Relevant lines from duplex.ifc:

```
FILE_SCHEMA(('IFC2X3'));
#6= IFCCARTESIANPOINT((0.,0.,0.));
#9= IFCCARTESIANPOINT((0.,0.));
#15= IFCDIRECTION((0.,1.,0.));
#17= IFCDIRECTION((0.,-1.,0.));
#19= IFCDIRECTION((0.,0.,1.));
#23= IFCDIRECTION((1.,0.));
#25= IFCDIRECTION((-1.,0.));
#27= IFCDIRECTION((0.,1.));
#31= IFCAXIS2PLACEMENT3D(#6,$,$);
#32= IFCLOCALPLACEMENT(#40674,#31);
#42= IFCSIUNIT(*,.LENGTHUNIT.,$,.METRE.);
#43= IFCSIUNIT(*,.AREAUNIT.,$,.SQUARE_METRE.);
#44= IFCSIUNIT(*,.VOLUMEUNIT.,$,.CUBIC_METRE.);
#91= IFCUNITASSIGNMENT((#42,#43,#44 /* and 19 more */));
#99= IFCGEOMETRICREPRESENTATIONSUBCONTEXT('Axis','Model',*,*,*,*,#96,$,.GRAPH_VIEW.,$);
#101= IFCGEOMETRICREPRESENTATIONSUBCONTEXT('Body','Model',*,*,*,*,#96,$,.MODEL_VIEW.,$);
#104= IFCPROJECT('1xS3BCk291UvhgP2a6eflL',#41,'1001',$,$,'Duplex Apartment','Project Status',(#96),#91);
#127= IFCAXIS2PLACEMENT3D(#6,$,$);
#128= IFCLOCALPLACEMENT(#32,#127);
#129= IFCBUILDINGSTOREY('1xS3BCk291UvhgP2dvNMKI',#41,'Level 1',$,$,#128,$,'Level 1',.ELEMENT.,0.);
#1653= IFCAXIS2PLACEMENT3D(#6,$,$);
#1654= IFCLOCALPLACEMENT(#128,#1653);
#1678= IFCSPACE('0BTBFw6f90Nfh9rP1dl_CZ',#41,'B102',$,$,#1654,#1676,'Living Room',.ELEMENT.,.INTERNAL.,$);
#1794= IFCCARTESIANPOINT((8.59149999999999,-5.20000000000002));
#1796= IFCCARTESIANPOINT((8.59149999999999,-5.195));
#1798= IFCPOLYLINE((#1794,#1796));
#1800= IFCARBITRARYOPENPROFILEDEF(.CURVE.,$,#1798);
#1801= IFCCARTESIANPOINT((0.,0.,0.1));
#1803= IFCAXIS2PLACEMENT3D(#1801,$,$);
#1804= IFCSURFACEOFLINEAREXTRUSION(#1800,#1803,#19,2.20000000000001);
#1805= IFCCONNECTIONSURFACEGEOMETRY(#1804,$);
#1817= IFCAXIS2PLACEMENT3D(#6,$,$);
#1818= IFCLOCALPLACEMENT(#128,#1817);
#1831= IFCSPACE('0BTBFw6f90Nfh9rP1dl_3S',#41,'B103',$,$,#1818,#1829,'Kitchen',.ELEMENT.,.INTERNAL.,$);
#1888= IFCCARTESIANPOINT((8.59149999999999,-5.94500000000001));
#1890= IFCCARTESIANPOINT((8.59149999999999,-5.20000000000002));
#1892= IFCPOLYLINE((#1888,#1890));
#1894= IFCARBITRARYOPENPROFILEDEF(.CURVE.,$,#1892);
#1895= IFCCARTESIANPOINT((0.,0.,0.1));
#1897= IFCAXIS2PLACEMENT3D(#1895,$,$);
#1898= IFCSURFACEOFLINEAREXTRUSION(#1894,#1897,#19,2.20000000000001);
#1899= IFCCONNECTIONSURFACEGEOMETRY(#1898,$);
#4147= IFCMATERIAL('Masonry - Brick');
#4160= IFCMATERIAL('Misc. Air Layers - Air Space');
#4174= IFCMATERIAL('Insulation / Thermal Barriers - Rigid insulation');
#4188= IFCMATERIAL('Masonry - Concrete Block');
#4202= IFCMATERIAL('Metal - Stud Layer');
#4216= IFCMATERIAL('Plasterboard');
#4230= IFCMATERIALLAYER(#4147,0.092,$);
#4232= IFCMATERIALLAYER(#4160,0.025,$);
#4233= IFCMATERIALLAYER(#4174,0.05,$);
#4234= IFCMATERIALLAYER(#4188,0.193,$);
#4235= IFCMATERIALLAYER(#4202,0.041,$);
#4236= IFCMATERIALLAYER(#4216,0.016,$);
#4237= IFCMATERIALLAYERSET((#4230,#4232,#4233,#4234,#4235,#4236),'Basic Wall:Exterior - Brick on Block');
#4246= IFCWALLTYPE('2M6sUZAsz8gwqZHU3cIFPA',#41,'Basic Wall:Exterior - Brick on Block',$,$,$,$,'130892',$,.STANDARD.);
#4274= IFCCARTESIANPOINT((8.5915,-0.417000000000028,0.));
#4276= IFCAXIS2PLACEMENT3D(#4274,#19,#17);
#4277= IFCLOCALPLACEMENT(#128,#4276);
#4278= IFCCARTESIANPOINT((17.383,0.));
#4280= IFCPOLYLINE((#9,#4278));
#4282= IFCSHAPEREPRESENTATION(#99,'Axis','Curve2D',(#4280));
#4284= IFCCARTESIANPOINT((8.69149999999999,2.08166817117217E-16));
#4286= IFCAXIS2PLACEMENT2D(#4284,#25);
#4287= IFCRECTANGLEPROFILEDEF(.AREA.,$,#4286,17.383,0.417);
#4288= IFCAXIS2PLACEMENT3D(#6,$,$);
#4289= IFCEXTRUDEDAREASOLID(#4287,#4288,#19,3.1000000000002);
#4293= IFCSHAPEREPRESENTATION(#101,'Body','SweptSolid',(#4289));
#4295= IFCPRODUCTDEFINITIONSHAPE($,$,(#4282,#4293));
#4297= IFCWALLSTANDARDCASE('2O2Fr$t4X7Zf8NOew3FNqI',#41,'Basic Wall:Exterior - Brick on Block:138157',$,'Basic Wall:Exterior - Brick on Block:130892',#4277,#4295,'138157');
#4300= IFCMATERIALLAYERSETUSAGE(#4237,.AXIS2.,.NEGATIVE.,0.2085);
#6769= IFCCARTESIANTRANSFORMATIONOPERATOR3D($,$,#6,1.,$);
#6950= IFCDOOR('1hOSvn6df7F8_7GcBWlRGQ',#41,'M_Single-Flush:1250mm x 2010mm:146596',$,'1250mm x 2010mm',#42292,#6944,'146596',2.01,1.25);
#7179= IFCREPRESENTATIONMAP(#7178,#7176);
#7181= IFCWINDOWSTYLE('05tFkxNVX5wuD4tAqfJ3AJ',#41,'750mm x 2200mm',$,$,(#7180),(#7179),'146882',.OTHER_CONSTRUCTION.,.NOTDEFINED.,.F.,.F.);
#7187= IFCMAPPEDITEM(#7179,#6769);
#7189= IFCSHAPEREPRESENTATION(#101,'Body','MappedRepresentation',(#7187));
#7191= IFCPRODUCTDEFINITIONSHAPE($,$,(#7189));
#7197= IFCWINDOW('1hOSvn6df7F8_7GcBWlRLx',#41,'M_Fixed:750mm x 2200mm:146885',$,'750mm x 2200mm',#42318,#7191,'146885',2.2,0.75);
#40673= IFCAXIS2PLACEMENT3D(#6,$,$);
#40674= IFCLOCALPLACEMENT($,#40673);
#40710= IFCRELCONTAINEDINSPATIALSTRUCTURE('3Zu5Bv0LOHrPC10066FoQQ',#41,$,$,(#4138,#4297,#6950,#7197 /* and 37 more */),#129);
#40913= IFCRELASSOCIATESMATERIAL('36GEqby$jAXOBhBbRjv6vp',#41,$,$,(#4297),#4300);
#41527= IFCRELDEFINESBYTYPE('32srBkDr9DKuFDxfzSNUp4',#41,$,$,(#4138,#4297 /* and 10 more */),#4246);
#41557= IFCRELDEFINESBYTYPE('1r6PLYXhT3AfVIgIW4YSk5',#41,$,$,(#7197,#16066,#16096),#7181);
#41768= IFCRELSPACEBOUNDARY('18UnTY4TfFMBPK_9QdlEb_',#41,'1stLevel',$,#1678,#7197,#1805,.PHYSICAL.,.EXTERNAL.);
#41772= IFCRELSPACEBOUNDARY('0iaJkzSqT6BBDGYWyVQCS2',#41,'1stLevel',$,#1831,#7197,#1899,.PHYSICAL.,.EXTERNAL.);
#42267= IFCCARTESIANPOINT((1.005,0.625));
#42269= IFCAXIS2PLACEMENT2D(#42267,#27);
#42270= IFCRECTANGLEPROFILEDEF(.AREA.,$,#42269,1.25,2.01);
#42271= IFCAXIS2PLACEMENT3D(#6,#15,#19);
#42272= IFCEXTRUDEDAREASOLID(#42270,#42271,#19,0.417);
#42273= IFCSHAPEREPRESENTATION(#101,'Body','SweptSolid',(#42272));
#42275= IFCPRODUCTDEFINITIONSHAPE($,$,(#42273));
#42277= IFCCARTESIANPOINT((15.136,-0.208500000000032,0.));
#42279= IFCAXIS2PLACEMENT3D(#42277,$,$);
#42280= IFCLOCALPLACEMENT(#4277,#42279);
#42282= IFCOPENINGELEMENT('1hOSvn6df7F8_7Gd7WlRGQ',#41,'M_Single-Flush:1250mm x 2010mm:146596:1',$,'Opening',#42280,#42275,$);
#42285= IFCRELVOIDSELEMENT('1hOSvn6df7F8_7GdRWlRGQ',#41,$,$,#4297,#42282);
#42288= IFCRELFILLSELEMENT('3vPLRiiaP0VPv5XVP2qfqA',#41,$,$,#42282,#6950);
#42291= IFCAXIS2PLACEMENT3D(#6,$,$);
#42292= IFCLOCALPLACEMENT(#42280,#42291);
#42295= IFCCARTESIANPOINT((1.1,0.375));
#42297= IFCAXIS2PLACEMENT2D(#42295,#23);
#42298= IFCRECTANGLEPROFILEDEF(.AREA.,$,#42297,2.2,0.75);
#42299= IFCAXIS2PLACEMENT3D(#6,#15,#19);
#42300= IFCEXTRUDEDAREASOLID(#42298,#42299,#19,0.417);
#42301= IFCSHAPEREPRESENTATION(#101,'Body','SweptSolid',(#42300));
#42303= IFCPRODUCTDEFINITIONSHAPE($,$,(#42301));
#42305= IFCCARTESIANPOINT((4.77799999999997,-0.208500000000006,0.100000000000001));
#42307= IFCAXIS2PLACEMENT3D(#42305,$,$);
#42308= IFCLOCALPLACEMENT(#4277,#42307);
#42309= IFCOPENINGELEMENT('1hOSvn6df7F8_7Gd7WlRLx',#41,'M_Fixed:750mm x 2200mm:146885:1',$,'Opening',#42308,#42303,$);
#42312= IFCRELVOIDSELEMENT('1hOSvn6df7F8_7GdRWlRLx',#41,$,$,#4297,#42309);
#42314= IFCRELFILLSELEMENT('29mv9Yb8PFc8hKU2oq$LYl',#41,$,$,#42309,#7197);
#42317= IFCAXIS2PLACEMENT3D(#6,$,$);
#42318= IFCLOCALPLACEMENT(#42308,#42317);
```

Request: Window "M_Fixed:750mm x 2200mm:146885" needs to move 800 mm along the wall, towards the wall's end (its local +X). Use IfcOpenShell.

```python
import numpy as np
import ifcopenshell
import ifcopenshell.api.geometry
import ifcopenshell.util.placement

model = ifcopenshell.open("duplex.ifc")

window = model.by_guid("1hOSvn6df7F8_7GcBWlRLx")
opening = window.FillsVoids[0].RelatingOpeningElement
wall = opening.VoidsElements[0].RelatingBuildingElement

wall_matrix = ifcopenshell.util.placement.get_local_placement(wall.ObjectPlacement)
shift = wall_matrix[:3, 0] * 0.8
before = ifcopenshell.util.placement.get_local_placement(window.ObjectPlacement)[:3, 3].copy()

# The window is placed relative to its opening, so it follows when the opening moves.
matrix = ifcopenshell.util.placement.get_local_placement(opening.ObjectPlacement)
matrix[:3, 3] += shift
ifcopenshell.api.geometry.edit_object_placement(
    model, product=opening, matrix=matrix, is_si=False, should_transform_children=True
)

# Space boundary surfaces are stored in each space's coordinates; move them too.
for rel in window.ProvidesBoundaries:
    if not rel.ConnectionGeometry:
        continue
    surface = rel.ConnectionGeometry.SurfaceOnRelatingElement
    space_matrix = ifcopenshell.util.placement.get_local_placement(rel.RelatingSpace.ObjectPlacement)
    point = np.array(surface.Position.Location.Coordinates) + space_matrix[:3, :3].T @ shift
    surface.Position = model.createIfcAxis2Placement3D(
        model.createIfcCartesianPoint(point.tolist()), surface.Position.Axis, surface.Position.RefDirection
    )

after = ifcopenshell.util.placement.get_local_placement(window.ObjectPlacement)[:3, 3]
print("window moved by", (after - before).round(3) + 0.0)

model.write("duplex_edited.ifc")
```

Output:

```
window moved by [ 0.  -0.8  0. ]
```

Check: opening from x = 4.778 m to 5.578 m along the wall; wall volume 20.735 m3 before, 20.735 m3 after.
